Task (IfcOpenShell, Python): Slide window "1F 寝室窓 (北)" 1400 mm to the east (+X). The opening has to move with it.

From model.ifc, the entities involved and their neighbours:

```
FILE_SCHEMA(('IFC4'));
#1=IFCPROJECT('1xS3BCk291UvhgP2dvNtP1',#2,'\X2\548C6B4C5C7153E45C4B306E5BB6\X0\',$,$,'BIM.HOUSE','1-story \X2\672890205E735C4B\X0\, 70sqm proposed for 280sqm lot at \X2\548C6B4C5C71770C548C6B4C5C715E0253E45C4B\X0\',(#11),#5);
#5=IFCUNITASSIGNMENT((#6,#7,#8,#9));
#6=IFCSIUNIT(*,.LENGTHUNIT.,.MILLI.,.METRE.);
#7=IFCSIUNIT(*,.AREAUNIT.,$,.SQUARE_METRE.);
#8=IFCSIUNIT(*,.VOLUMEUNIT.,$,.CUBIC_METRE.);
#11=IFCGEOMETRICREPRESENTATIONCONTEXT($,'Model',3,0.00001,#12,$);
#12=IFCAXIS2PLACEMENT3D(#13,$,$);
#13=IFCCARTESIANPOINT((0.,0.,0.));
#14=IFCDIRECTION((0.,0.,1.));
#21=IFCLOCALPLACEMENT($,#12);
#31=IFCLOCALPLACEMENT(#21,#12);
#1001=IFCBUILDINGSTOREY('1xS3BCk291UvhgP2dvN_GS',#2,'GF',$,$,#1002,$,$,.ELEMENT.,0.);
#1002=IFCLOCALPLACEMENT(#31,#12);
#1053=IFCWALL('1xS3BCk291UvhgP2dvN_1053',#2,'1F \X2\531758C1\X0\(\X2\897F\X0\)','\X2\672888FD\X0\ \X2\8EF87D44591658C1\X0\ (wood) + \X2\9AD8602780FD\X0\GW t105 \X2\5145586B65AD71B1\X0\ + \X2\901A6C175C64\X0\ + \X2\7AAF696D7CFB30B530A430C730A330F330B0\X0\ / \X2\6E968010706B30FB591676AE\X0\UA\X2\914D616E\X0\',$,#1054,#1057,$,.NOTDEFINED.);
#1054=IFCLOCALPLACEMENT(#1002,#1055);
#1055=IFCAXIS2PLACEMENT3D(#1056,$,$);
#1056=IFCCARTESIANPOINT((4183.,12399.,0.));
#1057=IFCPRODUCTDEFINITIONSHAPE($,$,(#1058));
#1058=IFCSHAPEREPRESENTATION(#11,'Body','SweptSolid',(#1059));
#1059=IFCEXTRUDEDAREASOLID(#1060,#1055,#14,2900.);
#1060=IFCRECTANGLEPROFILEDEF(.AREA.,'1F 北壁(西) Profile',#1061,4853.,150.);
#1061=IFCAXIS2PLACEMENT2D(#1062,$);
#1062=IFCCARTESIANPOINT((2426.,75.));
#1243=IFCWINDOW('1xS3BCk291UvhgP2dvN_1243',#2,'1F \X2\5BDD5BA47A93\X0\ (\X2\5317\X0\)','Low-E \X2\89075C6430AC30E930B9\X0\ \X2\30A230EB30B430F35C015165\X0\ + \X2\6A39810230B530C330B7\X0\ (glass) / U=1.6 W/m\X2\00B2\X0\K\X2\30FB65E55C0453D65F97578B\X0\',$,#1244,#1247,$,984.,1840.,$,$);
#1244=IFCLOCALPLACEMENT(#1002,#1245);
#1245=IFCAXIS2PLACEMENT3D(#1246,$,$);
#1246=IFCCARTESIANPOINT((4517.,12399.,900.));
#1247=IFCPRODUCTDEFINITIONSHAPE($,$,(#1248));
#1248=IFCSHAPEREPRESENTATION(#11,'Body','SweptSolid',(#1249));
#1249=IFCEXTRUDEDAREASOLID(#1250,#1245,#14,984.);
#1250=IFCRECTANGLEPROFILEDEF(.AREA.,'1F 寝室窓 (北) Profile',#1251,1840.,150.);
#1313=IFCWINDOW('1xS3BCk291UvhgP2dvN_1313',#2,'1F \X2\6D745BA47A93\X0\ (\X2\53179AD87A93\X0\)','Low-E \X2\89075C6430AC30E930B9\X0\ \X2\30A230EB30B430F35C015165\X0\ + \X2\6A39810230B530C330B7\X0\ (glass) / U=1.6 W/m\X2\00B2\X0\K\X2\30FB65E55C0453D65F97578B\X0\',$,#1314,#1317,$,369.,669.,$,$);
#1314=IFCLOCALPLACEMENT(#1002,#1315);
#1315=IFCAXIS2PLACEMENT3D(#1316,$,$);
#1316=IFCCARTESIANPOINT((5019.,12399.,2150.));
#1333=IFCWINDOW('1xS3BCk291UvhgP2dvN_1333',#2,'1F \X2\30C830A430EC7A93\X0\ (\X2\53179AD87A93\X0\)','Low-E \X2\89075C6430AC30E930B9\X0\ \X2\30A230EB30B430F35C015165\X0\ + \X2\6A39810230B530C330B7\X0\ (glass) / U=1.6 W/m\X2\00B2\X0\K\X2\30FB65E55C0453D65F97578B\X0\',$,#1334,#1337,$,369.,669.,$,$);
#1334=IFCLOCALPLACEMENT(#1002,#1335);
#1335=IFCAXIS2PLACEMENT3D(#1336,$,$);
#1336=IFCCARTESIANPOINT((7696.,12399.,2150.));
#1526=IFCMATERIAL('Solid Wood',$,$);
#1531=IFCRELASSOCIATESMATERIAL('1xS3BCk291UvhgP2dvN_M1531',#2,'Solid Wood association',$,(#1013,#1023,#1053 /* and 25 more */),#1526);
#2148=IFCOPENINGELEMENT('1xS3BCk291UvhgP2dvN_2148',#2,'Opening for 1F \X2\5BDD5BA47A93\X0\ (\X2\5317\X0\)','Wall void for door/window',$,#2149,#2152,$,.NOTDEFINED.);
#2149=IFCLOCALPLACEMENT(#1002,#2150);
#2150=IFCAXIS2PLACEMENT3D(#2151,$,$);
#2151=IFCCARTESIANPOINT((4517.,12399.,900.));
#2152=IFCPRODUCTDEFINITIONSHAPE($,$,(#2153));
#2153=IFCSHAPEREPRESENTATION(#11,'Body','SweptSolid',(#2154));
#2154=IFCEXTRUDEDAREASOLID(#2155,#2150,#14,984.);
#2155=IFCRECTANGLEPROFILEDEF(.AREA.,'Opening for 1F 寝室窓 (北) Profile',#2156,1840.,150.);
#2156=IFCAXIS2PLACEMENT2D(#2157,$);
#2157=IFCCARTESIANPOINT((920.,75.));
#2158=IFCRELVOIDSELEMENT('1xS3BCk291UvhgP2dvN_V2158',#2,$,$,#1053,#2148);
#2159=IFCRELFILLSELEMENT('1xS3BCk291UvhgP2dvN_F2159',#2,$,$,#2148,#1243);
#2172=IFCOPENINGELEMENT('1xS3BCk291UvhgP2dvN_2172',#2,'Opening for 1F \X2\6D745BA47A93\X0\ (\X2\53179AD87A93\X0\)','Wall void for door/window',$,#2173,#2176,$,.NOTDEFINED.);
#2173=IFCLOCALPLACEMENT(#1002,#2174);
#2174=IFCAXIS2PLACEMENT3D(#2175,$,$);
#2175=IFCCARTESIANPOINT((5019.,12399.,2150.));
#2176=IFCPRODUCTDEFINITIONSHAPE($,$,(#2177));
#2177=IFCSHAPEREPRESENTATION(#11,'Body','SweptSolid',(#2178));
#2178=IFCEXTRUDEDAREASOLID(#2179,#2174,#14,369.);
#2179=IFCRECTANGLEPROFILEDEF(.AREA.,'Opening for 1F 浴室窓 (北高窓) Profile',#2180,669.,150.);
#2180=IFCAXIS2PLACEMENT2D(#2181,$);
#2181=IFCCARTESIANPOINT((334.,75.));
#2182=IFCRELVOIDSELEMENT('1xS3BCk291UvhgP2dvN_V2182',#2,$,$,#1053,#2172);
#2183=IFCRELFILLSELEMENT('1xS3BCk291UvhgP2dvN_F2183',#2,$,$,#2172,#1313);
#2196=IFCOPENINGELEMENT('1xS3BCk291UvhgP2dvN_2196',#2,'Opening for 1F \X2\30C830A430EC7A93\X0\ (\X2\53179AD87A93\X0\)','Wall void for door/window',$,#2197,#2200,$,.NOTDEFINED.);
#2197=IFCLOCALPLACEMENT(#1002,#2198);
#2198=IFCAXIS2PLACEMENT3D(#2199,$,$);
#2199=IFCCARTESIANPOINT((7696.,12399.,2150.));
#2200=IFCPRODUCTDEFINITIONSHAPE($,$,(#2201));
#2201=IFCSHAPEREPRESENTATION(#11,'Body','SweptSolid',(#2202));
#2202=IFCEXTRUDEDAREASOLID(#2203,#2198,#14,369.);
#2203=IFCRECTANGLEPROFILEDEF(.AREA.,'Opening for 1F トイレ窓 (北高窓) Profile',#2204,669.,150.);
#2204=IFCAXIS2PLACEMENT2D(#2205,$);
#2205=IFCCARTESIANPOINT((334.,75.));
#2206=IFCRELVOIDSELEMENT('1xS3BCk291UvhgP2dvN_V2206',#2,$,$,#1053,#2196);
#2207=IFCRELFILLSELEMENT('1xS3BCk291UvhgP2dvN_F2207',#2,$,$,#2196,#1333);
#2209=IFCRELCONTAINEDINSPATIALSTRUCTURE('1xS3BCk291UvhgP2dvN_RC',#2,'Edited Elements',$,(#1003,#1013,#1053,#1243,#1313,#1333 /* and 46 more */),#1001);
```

```python
import ifcopenshell
import ifcopenshell.api.geometry
import ifcopenshell.util.placement

model = ifcopenshell.open("model.ifc")

window = model.by_id(1243)
opening = window.FillsVoids[0].RelatingOpeningElement
wall = opening.VoidsElements[0].RelatingBuildingElement

wall_matrix = ifcopenshell.util.placement.get_local_placement(wall.ObjectPlacement)
shift = wall_matrix[:3, 0] * 1400.0
before = ifcopenshell.util.placement.get_local_placement(window.ObjectPlacement)[:3, 3].copy()

# The window is not placed relative to its opening, so move both.
for product in (opening, window):
    matrix = ifcopenshell.util.placement.get_local_placement(product.ObjectPlacement)
    matrix[:3, 3] += shift
    ifcopenshell.api.geometry.edit_object_placement(model, product=product, matrix=matrix, is_si=False)

after = ifcopenshell.util.placement.get_local_placement(window.ObjectPlacement)[:3, 3]
print("window moved by", (after - before).round(3) + 0.0)

model.write("model_rev.ifc")
```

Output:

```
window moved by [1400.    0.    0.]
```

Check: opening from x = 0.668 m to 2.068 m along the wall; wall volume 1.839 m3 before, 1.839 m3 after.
